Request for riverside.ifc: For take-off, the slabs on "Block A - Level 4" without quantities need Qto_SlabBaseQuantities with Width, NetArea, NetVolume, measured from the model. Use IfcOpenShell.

First a look at what the model holds.

```python
import ifcopenshell
import ifcopenshell.util.element
import ifcopenshell.util.unit

model = ifcopenshell.open("riverside.ifc")
print(model.schema)
for unit_type in ("LENGTHUNIT", "AREAUNIT", "VOLUMEUNIT"):
    print(unit_type, ifcopenshell.util.unit.calculate_unit_scale(model, unit_type))
storey = next(s for s in model.by_type("IfcBuildingStorey") if s.Name == "Block A - Level 4")
slabs = [e for e in ifcopenshell.util.element.get_decomposition(storey) if e.is_a("IfcSlab")]
for e in sorted(slabs, key=lambda e: e.id()):
    print(e.id(), e.is_a(), e.Name, list(ifcopenshell.util.element.get_psets(e, qtos_only=True)), sep=" | ")
```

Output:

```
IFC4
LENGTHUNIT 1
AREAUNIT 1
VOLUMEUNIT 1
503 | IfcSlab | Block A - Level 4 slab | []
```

```python
import ifcopenshell
import ifcopenshell.api.pset
import ifcopenshell.geom
import ifcopenshell.util.element
import ifcopenshell.util.shape
import ifcopenshell.util.unit

model = ifcopenshell.open("riverside.ifc")
unit_scale = ifcopenshell.util.unit.calculate_unit_scale(model)
area_scale = ifcopenshell.util.unit.calculate_unit_scale(model, "AREAUNIT")
volume_scale = ifcopenshell.util.unit.calculate_unit_scale(model, "VOLUMEUNIT")
settings = ifcopenshell.geom.settings()

storey = next(s for s in model.by_type("IfcBuildingStorey") if s.Name == "Block A - Level 4")
slabs = [e for e in ifcopenshell.util.element.get_decomposition(storey) if e.is_a("IfcSlab")]

for e in sorted(slabs, key=lambda e: e.id()):
    if ifcopenshell.util.element.get_psets(e, qtos_only=True, should_inherit=False):
        continue
    # Geometry comes back in metres, in the element's own axes.
    shape = ifcopenshell.geom.create_shape(settings, e)
    values = {
        "Width": ifcopenshell.util.shape.get_z(shape.geometry) / unit_scale,
        "NetArea": ifcopenshell.util.shape.get_footprint_area(shape.geometry) / area_scale,
        "NetVolume": ifcopenshell.util.shape.get_volume(shape.geometry) / volume_scale,
    }
    qto = ifcopenshell.api.pset.add_qto(model, product=e, name="Qto_SlabBaseQuantities")
    ifcopenshell.api.pset.edit_qto(model, qto=qto, properties=values)
    print(e.id(), {k: round(v, 3) for k, v in values.items()})

model.write("riverside_edited.ifc")
```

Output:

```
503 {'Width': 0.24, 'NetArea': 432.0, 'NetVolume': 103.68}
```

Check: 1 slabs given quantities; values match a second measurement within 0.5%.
